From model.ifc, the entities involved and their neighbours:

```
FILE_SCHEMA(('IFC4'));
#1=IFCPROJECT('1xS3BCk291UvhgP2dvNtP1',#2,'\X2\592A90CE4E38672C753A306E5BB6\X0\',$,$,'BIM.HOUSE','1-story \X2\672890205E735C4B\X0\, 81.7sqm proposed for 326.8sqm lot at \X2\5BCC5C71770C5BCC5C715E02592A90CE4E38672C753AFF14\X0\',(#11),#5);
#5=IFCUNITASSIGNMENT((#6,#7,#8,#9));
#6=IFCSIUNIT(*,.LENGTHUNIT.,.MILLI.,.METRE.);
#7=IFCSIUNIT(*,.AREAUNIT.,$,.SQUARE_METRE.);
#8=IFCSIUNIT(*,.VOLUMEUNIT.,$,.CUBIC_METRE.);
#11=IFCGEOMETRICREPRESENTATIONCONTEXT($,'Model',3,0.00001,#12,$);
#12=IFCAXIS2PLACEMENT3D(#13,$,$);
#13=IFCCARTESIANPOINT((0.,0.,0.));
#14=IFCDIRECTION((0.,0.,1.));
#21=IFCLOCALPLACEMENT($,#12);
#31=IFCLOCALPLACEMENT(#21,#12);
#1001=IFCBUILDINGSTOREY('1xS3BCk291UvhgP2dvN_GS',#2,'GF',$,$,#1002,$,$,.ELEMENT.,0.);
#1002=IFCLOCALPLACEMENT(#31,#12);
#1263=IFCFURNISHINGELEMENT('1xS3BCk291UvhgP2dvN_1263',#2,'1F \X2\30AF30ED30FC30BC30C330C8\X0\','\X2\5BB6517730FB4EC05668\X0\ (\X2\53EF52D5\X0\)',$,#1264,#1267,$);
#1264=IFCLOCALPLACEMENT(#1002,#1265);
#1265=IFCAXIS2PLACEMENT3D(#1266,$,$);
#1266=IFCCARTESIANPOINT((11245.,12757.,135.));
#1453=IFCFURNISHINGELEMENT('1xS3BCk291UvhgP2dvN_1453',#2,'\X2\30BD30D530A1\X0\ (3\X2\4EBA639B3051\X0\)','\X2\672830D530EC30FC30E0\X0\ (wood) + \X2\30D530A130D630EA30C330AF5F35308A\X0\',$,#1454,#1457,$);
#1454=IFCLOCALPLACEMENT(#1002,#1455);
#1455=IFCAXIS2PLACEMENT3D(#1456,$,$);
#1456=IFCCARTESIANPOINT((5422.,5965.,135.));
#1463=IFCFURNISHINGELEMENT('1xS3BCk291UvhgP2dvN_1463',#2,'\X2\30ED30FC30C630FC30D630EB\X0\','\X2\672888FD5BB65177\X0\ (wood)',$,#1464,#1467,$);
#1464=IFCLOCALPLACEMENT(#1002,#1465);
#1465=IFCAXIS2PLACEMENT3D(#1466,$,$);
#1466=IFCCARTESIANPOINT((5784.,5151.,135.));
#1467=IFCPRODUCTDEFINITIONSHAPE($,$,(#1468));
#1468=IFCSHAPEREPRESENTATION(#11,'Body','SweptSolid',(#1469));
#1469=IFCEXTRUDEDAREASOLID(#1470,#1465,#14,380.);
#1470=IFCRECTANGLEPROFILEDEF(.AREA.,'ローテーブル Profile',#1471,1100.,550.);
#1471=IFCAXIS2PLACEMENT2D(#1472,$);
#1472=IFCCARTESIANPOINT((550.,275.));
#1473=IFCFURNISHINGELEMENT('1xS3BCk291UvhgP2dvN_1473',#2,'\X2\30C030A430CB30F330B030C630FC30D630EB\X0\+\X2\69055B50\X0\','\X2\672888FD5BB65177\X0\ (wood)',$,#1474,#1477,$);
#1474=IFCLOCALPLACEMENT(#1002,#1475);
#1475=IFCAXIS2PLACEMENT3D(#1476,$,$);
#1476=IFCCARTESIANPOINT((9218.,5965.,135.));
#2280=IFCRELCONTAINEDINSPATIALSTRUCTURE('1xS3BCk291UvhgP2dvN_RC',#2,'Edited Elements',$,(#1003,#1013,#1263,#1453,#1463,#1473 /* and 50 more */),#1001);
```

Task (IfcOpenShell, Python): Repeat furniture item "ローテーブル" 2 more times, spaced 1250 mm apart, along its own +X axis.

```python
import ifcopenshell
import ifcopenshell.api.geometry
import ifcopenshell.api.root
import ifcopenshell.util.element
import ifcopenshell.util.placement

model = ifcopenshell.open("model.ifc")


def reuse_history(source, copy):
    """copy_class also copies each property set's owner history, people and application; keep the originals."""
    for rel in copy.IsDefinedBy:
        if rel.is_a("IfcRelDefinesByProperties") and (history := rel.RelatingPropertyDefinition.OwnerHistory):
            rel.RelatingPropertyDefinition.OwnerHistory = source.OwnerHistory
            ifcopenshell.util.element.remove_deep2(model, history)


source = model.by_id(1463)
base = ifcopenshell.util.placement.get_local_placement(source.ObjectPlacement)
step = base[:3, 0] * 1250.0

for i in range(1, 3):
    copy = ifcopenshell.api.root.copy_class(model, product=source)
    copy.Representation = ifcopenshell.util.element.copy_deep(
        model, source.Representation, exclude=["IfcGeometricRepresentationContext", "IfcRepresentationMap"]
    )
    reuse_history(source, copy)
    matrix = base.copy()
    matrix[:3, 3] += i * step
    print("added at", matrix[:3, 3].round(3) + 0.0)
    ifcopenshell.api.geometry.edit_object_placement(model, product=copy, matrix=matrix, is_si=False)

model.write("model-out.ifc")
```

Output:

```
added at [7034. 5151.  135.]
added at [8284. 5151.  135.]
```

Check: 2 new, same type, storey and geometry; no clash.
